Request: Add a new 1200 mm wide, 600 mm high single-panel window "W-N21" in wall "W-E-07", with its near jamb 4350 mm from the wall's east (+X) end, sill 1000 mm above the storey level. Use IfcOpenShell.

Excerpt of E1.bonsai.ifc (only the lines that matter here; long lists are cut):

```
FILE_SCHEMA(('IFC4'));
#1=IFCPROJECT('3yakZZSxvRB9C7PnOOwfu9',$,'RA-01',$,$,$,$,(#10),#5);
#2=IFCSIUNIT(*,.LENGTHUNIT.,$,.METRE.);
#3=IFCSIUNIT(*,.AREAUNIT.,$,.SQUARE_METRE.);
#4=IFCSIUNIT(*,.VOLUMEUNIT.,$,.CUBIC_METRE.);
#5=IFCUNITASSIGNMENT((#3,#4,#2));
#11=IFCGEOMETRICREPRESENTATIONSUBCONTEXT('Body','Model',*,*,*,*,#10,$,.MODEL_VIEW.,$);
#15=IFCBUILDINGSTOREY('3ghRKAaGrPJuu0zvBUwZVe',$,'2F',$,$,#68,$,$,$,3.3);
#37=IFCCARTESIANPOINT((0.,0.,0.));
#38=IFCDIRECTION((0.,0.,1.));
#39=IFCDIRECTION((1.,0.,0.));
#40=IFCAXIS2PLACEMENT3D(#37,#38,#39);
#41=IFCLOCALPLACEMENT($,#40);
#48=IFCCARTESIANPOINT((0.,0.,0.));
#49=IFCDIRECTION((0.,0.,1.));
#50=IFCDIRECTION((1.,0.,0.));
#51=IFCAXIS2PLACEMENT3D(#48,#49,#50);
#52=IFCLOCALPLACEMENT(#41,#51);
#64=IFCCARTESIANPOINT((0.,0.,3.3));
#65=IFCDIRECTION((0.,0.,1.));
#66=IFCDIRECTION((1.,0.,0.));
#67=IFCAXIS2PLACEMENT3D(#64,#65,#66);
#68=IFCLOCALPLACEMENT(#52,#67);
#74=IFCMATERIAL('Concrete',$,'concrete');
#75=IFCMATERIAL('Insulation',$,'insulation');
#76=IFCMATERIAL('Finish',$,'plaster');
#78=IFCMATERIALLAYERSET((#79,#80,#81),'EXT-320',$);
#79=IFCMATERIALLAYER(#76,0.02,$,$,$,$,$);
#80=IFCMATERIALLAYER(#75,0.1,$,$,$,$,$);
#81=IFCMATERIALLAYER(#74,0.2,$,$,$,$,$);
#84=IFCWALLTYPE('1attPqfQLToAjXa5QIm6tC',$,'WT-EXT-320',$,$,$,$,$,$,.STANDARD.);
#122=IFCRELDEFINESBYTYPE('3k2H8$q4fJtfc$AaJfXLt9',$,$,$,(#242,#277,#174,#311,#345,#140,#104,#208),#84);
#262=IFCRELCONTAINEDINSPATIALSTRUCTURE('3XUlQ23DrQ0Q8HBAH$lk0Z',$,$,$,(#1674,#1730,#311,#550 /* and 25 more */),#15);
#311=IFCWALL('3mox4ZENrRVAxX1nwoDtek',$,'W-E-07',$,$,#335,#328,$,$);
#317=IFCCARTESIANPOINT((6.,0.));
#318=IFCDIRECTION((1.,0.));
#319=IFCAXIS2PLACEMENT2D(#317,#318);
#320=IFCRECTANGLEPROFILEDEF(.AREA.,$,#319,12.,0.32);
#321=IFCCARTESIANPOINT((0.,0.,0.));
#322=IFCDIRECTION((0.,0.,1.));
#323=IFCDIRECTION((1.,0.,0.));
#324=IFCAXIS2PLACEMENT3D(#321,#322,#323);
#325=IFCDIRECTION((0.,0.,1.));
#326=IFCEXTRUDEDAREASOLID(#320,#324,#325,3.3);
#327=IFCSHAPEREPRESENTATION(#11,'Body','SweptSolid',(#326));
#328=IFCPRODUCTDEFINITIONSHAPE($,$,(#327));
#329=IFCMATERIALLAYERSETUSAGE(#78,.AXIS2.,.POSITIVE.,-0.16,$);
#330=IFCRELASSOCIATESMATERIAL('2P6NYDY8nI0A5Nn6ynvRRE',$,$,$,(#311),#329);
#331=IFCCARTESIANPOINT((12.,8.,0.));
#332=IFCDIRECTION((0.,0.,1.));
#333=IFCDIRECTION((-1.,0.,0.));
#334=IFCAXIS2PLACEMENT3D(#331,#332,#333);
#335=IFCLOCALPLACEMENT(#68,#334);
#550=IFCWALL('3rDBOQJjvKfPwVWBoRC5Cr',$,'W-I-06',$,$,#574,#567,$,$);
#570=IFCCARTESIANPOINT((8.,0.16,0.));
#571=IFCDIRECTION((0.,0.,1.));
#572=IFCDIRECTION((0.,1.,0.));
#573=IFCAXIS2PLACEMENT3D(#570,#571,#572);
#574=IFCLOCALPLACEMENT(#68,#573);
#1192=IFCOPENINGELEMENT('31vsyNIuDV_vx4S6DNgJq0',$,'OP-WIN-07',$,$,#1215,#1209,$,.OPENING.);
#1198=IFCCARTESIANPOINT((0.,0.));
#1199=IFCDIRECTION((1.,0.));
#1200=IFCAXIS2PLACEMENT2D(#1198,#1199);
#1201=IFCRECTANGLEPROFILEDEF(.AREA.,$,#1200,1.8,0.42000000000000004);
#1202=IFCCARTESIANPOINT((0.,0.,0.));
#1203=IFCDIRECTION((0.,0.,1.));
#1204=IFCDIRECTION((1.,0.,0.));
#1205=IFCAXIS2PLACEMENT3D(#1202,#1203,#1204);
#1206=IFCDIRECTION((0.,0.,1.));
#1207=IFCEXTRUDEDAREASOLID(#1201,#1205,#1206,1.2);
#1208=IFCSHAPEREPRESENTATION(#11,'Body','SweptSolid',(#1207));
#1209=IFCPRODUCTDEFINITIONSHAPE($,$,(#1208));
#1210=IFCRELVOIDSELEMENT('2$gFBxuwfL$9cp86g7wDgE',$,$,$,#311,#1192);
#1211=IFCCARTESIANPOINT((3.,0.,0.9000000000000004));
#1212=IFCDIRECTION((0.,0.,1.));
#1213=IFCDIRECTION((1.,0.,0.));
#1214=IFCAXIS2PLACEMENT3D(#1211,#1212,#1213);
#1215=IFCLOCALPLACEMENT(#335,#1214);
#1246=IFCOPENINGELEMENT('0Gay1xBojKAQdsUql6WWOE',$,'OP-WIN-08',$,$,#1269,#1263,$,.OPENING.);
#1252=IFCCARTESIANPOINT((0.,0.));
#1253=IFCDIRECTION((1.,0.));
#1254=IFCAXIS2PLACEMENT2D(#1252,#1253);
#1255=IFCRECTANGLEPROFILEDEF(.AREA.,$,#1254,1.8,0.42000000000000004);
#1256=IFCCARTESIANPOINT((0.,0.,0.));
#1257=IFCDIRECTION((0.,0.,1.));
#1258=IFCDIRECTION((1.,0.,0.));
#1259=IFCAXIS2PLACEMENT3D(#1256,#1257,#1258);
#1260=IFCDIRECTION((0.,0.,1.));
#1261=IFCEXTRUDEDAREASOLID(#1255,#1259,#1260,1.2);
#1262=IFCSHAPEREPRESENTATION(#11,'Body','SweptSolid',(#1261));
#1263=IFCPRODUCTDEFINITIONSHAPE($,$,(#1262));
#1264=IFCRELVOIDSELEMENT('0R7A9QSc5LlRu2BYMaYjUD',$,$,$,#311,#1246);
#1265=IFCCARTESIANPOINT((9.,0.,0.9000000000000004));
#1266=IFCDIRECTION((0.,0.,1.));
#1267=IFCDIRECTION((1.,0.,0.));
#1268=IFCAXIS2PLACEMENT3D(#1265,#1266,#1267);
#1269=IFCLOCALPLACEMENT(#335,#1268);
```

```python
import numpy as np
import ifcopenshell
import ifcopenshell.api.feature
import ifcopenshell.api.geometry
import ifcopenshell.api.root
import ifcopenshell.api.spatial
import ifcopenshell.geom
import ifcopenshell.util.element
import ifcopenshell.util.placement
import ifcopenshell.util.representation
import ifcopenshell.util.shape
import ifcopenshell.util.unit

model = ifcopenshell.open("E1.bonsai.ifc")
unit_scale = ifcopenshell.util.unit.calculate_unit_scale(model)
settings = ifcopenshell.geom.settings()


def volume(element):
    """Net volume in cubic metres, openings subtracted."""
    shape = ifcopenshell.geom.create_shape(settings, element)
    return ifcopenshell.util.shape.get_volume(shape.geometry)


wall = model.by_id(311)
storey = ifcopenshell.util.element.get_container(wall, ifc_class="IfcBuildingStorey")
context = ifcopenshell.util.representation.get_context(model, "Model", "Body", "MODEL_VIEW")
before = volume(wall)

width, height, from_end, sill = 1.2, 0.6, 4.35, 1  # metres

# The wall runs along its own X axis, and the end named is its -X end.
wall_shape = ifcopenshell.geom.create_shape(settings, wall)
x, y, z = ifcopenshell.util.shape.get_vertices(wall_shape.geometry).T
start = x.min() + from_end
face, thickness = float(y.min()), float(y.max() - y.min())
wall_matrix = ifcopenshell.util.placement.get_local_placement(wall.ObjectPlacement)
level = ifcopenshell.util.placement.get_local_placement(storey.ObjectPlacement)[2, 3]


def in_wall(x, y):
    """Placement at x, y metres in the wall's axes, at sill height."""
    matrix = wall_matrix.copy()
    matrix[:, 3] = wall_matrix @ np.array([x / unit_scale, y / unit_scale, 0.0, 1.0])
    matrix[2, 3] = level + sill / unit_scale
    return matrix


# Opening: a box that overshoots both wall faces by 50 mm.
opening = ifcopenshell.api.root.create_entity(model, ifc_class="IfcOpeningElement", predefined_type="OPENING")
box = ifcopenshell.api.geometry.add_wall_representation(
    model, context=context, length=width, height=height, thickness=thickness + 0.1
)
ifcopenshell.api.geometry.assign_representation(model, product=opening, representation=box)
ifcopenshell.api.geometry.edit_object_placement(model, product=opening, matrix=in_wall(start, face - 0.05), is_si=False)
ifcopenshell.api.feature.add_feature(model, feature=opening, element=wall)

window = ifcopenshell.api.root.create_entity(model, ifc_class="IfcWindow", name="W-N21", predefined_type="WINDOW")
window.OverallWidth, window.OverallHeight = width / unit_scale, height / unit_scale
window.PartitioningType = "SINGLE_PANEL"
body = ifcopenshell.api.geometry.add_window_representation(
    model,
    context=context,
    overall_width=window.OverallWidth,
    overall_height=window.OverallHeight,
    partition_type="SINGLE_PANEL",
)
ifcopenshell.api.geometry.assign_representation(model, product=window, representation=body)
ifcopenshell.api.spatial.assign_container(model, products=[window], relating_structure=storey)
ifcopenshell.api.feature.add_filling(model, opening=opening, element=window)

# Centre the window in the wall's thickness.
ifcopenshell.api.geometry.edit_object_placement(model, product=window, matrix=in_wall(start, face), is_si=False)
window_shape = ifcopenshell.geom.create_shape(settings, window)
depth = ifcopenshell.util.shape.get_vertices(window_shape.geometry)[:, 1]
offset = face + thickness / 2 - (depth.min() + depth.max()) / 2
ifcopenshell.api.geometry.edit_object_placement(model, product=window, matrix=in_wall(start, offset), is_si=False)

after = volume(wall)

print(f"wall volume {before:.3f} -> {after:.3f} m3")

model.write("E1.bonsai_rev.ifc")
```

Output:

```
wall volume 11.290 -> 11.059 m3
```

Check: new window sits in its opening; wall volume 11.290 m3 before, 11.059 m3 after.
